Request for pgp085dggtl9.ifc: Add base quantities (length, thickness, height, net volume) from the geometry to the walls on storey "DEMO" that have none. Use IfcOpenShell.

First a look at what the model holds.

```python
import ifcopenshell
import ifcopenshell.util.element
import ifcopenshell.util.unit

model = ifcopenshell.open("pgp085dggtl9.ifc")
print(model.schema)
for unit_type in ("LENGTHUNIT", "AREAUNIT", "VOLUMEUNIT"):
    print(unit_type, ifcopenshell.util.unit.calculate_unit_scale(model, unit_type))
storey = next(s for s in model.by_type("IfcBuildingStorey") if s.Name == "DEMO")
walls = [e for e in ifcopenshell.util.element.get_decomposition(storey) if e.is_a("IfcWall")]
for e in sorted(walls, key=lambda e: e.id()):
    print(e.id(), e.is_a(), e.Name, list(ifcopenshell.util.element.get_psets(e, qtos_only=True)), sep=" | ")
```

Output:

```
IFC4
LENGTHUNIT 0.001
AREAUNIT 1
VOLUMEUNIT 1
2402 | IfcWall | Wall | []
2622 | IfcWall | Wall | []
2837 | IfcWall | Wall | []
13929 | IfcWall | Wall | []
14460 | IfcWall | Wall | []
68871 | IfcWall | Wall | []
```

```python
import ifcopenshell
import ifcopenshell.api.pset
import ifcopenshell.geom
import ifcopenshell.util.element
import ifcopenshell.util.shape
import ifcopenshell.util.unit

model = ifcopenshell.open("pgp085dggtl9.ifc")
unit_scale = ifcopenshell.util.unit.calculate_unit_scale(model)
volume_scale = ifcopenshell.util.unit.calculate_unit_scale(model, "VOLUMEUNIT")
settings = ifcopenshell.geom.settings()

storey = next(s for s in model.by_type("IfcBuildingStorey") if s.Name == "DEMO")
walls = [e for e in ifcopenshell.util.element.get_decomposition(storey) if e.is_a("IfcWall")]

for e in sorted(walls, key=lambda e: e.id()):
    if ifcopenshell.util.element.get_psets(e, qtos_only=True, should_inherit=False):
        continue
    # Geometry comes back in metres, in the element's own axes.
    shape = ifcopenshell.geom.create_shape(settings, e)
    values = {
        "Length": ifcopenshell.util.shape.get_x(shape.geometry) / unit_scale,
        "Width": ifcopenshell.util.shape.get_y(shape.geometry) / unit_scale,
        "Height": ifcopenshell.util.shape.get_z(shape.geometry) / unit_scale,
        "NetVolume": ifcopenshell.util.shape.get_volume(shape.geometry) / volume_scale,
    }
    qto = ifcopenshell.api.pset.add_qto(model, product=e, name="Qto_WallBaseQuantities")
    ifcopenshell.api.pset.edit_qto(model, qto=qto, properties=values)
    print(e.id(), {k: round(v, 3) for k, v in values.items()})

model.write("pgp085dggtl9_edited.ifc")
```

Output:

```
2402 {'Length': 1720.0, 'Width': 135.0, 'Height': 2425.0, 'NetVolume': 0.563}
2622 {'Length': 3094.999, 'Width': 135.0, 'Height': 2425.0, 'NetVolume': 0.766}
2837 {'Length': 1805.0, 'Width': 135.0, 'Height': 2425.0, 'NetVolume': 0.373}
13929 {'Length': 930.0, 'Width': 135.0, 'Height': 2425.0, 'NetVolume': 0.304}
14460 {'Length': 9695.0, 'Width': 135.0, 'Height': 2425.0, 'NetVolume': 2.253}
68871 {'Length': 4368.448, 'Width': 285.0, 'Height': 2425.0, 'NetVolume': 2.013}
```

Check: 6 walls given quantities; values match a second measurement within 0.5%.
